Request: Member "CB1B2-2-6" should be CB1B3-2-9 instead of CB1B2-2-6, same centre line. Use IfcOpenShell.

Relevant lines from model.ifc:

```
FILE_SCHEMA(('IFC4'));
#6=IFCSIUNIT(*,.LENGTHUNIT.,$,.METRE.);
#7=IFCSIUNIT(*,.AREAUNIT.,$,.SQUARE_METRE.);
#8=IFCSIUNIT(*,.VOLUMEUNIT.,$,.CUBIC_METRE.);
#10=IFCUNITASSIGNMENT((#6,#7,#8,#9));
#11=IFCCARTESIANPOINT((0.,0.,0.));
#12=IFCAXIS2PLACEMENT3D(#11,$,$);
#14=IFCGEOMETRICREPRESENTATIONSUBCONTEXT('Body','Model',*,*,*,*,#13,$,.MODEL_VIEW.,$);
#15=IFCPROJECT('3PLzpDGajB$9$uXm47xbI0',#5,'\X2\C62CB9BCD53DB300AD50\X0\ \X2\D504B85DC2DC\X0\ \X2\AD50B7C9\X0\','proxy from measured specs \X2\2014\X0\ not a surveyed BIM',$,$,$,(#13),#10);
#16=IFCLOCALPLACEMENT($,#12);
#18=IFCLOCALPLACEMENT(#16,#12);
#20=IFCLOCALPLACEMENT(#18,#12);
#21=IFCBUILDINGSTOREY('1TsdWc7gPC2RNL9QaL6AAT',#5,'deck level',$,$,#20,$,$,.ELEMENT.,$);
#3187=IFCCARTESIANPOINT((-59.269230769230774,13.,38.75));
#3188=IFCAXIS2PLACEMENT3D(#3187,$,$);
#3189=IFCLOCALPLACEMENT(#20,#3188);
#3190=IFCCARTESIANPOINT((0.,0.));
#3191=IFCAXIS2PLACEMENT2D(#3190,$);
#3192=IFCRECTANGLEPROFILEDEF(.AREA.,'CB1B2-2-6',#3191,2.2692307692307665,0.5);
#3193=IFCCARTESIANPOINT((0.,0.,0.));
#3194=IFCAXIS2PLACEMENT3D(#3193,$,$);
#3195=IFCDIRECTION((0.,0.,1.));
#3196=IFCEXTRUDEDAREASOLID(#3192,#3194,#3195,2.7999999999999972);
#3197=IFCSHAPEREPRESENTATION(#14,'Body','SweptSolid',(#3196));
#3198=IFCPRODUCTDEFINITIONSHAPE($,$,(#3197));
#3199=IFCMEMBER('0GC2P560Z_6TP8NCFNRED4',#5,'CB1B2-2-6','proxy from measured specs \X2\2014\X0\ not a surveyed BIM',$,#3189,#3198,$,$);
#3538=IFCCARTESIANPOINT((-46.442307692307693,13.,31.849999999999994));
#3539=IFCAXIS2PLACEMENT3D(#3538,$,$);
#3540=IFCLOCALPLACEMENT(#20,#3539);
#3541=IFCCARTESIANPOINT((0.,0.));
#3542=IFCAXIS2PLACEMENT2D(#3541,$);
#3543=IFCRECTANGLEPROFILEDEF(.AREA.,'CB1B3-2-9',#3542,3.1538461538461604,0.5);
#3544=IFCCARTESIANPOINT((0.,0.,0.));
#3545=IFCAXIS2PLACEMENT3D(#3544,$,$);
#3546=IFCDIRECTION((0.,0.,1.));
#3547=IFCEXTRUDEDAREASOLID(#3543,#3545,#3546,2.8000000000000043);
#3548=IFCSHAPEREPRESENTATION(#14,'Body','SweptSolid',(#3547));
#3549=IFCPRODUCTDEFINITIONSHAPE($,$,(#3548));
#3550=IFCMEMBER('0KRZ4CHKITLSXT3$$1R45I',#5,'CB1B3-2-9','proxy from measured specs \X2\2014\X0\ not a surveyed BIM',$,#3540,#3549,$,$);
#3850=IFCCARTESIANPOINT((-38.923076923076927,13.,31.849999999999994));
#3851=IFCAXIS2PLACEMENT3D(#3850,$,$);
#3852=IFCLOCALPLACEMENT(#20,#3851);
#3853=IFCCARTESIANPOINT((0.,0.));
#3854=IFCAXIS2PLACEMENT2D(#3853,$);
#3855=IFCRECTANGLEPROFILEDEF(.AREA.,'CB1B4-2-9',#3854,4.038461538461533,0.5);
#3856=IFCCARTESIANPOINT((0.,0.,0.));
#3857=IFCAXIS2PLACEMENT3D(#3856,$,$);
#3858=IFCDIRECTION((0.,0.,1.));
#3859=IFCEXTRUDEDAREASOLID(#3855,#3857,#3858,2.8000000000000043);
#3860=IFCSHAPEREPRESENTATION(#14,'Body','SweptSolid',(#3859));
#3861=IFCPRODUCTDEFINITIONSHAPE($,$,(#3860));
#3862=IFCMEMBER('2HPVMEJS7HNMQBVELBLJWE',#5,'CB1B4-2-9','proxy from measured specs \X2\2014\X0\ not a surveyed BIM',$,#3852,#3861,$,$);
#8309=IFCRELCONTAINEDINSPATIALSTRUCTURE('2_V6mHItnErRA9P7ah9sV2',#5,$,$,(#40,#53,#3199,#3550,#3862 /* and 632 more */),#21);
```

```python
import ifcopenshell
import ifcopenshell.util.element
import ifcopenshell.util.representation

model = ifcopenshell.open("model.ifc")

member = model.by_guid("0GC2P560Z_6TP8NCFNRED4")
source = next(p for p in model.by_type("IfcRectangleProfileDef") if p.ProfileName == "CB1B3-2-9")

body = ifcopenshell.util.representation.get_representation(member, "Model", "Body")
solid = body.Items[0]
old_profile = solid.SweptArea

# Copy the section's sizes but keep this member's own profile position.
profile = ifcopenshell.util.element.copy(model, source)
profile.Position = old_profile.Position
solid.SweptArea = profile
if not model.get_total_inverses(old_profile):
    ifcopenshell.util.element.remove_deep2(model, old_profile)
member.Name = member.Name.replace("CB1B2-2-6", "CB1B3-2-9")

print(solid.SweptArea)

model.write("model_v2.ifc")
```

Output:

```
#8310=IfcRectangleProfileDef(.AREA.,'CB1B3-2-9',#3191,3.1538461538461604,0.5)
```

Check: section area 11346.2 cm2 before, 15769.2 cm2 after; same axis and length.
